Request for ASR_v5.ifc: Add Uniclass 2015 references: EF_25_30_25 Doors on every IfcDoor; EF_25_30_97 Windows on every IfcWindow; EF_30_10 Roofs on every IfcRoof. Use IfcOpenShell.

First a look at what the model holds.

```python
import ifcopenshell

model = ifcopenshell.open("ASR_v5.ifc")
print(model.schema)
print("classifications:", [c.Name for c in model.by_type("IfcClassification")])
for ifc_class in ("IfcDoor", "IfcRoof", "IfcStair", "IfcWall", "IfcWindow"):
    print(ifc_class, len(model.by_type(ifc_class)))
```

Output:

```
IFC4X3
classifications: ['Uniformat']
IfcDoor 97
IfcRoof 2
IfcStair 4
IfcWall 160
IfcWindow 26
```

```python
import ifcopenshell
import ifcopenshell.api.classification

model = ifcopenshell.open("ASR_v5.ifc")

system = ifcopenshell.api.classification.add_classification(model, classification="Uniclass 2015")

codes = {
    "IfcDoor": ("EF_25_30_25", "Doors"),
    "IfcWindow": ("EF_25_30_97", "Windows"),
    "IfcRoof": ("EF_30_10", "Roofs"),
}
for ifc_class, (code, name) in codes.items():
    products = model.by_type(ifc_class)
    ifcopenshell.api.classification.add_reference(
        model, products=products, classification=system, identification=code, name=name
    )
    print(code, len(products))

model.write("ASR_v5_updated.ifc")
```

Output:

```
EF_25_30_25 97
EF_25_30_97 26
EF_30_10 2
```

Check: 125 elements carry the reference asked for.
